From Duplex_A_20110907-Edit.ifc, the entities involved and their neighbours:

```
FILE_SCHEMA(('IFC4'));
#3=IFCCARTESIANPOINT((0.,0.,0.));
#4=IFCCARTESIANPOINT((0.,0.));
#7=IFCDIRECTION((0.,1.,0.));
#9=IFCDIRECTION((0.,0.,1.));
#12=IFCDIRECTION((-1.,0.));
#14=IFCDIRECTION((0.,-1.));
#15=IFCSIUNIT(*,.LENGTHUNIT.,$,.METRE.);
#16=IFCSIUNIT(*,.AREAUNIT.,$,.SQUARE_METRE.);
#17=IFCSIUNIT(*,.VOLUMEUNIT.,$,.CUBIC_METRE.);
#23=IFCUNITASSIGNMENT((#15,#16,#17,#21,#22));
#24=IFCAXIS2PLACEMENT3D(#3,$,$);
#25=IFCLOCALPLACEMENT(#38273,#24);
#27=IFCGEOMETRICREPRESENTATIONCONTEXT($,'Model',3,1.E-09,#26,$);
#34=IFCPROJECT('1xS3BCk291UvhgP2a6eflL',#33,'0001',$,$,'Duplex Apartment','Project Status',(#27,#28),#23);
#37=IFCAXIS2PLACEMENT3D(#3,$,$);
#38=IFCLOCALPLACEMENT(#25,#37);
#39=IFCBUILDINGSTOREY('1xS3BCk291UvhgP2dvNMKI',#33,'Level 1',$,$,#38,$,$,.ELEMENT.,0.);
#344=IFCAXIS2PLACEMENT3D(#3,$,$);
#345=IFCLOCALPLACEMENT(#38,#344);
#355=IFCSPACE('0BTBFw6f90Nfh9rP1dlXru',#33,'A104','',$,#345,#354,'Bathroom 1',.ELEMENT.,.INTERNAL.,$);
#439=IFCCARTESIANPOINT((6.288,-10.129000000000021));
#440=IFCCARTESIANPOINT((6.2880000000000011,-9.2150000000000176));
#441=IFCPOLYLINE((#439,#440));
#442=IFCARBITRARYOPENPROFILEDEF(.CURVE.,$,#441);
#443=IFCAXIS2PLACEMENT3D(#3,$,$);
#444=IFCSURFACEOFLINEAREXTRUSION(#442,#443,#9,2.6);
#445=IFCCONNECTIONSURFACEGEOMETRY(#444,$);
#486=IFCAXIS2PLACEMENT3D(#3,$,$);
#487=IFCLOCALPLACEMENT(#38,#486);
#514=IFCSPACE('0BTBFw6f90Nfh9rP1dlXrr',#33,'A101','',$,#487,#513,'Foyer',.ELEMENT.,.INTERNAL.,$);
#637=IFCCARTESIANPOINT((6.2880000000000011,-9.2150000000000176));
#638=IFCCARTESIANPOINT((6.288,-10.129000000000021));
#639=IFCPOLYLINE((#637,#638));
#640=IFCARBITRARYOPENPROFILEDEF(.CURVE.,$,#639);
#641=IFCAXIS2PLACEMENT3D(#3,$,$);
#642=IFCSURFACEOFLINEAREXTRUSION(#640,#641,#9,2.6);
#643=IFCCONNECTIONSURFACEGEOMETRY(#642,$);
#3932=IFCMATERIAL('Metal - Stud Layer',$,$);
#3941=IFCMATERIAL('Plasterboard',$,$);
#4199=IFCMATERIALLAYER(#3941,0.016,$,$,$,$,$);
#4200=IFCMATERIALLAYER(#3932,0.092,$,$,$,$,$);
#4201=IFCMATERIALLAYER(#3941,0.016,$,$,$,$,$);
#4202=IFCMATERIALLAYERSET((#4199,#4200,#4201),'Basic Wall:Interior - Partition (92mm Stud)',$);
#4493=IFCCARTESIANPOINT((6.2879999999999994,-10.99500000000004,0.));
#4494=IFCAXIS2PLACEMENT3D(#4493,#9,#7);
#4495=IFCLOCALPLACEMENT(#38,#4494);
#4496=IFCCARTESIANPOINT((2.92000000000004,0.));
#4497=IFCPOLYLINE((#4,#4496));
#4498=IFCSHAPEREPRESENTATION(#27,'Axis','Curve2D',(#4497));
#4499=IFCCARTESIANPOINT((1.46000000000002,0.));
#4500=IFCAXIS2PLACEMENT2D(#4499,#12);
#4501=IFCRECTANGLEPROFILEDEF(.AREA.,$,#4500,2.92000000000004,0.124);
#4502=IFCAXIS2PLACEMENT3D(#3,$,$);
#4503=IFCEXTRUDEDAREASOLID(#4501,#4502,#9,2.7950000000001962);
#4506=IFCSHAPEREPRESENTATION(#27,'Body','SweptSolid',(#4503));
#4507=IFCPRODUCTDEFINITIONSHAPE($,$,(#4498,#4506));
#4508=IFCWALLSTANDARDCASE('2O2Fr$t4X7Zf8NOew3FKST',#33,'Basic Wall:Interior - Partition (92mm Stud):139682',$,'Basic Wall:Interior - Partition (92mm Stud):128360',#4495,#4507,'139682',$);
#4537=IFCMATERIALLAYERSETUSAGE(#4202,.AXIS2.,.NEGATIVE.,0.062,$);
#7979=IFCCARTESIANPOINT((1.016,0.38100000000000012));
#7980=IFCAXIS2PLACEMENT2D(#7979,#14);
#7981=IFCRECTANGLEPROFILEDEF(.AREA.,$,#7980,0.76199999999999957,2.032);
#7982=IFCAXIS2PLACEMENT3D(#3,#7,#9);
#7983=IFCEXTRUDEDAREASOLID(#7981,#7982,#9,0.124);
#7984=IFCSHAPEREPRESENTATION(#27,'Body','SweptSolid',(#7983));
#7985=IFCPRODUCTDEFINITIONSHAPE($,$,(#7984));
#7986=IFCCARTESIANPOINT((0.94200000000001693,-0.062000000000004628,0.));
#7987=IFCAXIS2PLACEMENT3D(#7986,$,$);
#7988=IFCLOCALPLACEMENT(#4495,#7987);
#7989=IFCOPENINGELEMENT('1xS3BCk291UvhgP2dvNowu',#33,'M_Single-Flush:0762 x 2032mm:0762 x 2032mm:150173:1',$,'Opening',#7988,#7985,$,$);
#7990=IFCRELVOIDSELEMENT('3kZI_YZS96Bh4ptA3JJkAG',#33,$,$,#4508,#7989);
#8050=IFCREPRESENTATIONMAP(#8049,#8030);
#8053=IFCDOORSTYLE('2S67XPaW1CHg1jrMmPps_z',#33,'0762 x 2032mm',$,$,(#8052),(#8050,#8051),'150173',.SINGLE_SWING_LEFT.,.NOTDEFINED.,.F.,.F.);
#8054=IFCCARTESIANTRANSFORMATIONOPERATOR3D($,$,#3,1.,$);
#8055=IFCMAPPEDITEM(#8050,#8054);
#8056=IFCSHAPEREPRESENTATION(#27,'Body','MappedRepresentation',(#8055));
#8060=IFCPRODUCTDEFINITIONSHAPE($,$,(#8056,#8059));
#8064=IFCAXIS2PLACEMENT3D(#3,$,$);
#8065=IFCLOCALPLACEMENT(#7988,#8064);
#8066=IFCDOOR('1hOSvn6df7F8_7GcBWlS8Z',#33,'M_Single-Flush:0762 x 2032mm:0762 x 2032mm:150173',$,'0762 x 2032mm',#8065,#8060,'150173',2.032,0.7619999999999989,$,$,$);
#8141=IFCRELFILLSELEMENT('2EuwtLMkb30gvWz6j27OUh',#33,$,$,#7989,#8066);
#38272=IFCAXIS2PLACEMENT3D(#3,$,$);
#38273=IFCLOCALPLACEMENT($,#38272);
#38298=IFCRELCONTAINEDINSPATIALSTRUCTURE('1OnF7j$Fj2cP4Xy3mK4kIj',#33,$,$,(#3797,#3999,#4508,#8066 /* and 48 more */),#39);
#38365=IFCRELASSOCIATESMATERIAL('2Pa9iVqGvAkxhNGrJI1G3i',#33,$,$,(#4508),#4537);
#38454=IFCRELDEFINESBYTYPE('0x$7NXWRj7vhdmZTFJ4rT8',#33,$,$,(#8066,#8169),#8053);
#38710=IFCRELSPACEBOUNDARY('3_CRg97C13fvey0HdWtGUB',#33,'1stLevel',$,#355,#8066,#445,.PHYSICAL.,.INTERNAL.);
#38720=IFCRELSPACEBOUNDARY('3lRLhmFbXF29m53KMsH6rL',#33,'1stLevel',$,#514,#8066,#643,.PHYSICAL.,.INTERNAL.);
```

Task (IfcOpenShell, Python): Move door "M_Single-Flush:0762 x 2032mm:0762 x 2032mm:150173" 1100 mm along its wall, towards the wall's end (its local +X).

```python
import numpy as np
import ifcopenshell
import ifcopenshell.api.geometry
import ifcopenshell.util.placement

model = ifcopenshell.open("Duplex_A_20110907-Edit.ifc")

door = model.by_guid("1hOSvn6df7F8_7GcBWlS8Z")
opening = door.FillsVoids[0].RelatingOpeningElement
wall = opening.VoidsElements[0].RelatingBuildingElement

wall_matrix = ifcopenshell.util.placement.get_local_placement(wall.ObjectPlacement)
shift = wall_matrix[:3, 0] * 1.1
before = ifcopenshell.util.placement.get_local_placement(door.ObjectPlacement)[:3, 3].copy()

# The door is placed relative to its opening, so it follows when the opening moves.
matrix = ifcopenshell.util.placement.get_local_placement(opening.ObjectPlacement)
matrix[:3, 3] += shift
ifcopenshell.api.geometry.edit_object_placement(
    model, product=opening, matrix=matrix, is_si=False, should_transform_children=True
)

# Space boundary surfaces are stored in each space's coordinates; move them too.
for rel in door.ProvidesBoundaries:
    if not rel.ConnectionGeometry:
        continue
    surface = rel.ConnectionGeometry.SurfaceOnRelatingElement
    space_matrix = ifcopenshell.util.placement.get_local_placement(rel.RelatingSpace.ObjectPlacement)
    point = np.array(surface.Position.Location.Coordinates) + space_matrix[:3, :3].T @ shift
    surface.Position = model.createIfcAxis2Placement3D(
        model.createIfcCartesianPoint(point.tolist()), surface.Position.Axis, surface.Position.RefDirection
    )

after = ifcopenshell.util.placement.get_local_placement(door.ObjectPlacement)[:3, 3]
print("door moved by", (after - before).round(3) + 0.0)

model.write("Duplex_A_20110907-Edit_edited.ifc")
```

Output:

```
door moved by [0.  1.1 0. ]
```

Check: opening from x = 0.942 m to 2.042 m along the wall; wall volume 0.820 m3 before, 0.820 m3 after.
